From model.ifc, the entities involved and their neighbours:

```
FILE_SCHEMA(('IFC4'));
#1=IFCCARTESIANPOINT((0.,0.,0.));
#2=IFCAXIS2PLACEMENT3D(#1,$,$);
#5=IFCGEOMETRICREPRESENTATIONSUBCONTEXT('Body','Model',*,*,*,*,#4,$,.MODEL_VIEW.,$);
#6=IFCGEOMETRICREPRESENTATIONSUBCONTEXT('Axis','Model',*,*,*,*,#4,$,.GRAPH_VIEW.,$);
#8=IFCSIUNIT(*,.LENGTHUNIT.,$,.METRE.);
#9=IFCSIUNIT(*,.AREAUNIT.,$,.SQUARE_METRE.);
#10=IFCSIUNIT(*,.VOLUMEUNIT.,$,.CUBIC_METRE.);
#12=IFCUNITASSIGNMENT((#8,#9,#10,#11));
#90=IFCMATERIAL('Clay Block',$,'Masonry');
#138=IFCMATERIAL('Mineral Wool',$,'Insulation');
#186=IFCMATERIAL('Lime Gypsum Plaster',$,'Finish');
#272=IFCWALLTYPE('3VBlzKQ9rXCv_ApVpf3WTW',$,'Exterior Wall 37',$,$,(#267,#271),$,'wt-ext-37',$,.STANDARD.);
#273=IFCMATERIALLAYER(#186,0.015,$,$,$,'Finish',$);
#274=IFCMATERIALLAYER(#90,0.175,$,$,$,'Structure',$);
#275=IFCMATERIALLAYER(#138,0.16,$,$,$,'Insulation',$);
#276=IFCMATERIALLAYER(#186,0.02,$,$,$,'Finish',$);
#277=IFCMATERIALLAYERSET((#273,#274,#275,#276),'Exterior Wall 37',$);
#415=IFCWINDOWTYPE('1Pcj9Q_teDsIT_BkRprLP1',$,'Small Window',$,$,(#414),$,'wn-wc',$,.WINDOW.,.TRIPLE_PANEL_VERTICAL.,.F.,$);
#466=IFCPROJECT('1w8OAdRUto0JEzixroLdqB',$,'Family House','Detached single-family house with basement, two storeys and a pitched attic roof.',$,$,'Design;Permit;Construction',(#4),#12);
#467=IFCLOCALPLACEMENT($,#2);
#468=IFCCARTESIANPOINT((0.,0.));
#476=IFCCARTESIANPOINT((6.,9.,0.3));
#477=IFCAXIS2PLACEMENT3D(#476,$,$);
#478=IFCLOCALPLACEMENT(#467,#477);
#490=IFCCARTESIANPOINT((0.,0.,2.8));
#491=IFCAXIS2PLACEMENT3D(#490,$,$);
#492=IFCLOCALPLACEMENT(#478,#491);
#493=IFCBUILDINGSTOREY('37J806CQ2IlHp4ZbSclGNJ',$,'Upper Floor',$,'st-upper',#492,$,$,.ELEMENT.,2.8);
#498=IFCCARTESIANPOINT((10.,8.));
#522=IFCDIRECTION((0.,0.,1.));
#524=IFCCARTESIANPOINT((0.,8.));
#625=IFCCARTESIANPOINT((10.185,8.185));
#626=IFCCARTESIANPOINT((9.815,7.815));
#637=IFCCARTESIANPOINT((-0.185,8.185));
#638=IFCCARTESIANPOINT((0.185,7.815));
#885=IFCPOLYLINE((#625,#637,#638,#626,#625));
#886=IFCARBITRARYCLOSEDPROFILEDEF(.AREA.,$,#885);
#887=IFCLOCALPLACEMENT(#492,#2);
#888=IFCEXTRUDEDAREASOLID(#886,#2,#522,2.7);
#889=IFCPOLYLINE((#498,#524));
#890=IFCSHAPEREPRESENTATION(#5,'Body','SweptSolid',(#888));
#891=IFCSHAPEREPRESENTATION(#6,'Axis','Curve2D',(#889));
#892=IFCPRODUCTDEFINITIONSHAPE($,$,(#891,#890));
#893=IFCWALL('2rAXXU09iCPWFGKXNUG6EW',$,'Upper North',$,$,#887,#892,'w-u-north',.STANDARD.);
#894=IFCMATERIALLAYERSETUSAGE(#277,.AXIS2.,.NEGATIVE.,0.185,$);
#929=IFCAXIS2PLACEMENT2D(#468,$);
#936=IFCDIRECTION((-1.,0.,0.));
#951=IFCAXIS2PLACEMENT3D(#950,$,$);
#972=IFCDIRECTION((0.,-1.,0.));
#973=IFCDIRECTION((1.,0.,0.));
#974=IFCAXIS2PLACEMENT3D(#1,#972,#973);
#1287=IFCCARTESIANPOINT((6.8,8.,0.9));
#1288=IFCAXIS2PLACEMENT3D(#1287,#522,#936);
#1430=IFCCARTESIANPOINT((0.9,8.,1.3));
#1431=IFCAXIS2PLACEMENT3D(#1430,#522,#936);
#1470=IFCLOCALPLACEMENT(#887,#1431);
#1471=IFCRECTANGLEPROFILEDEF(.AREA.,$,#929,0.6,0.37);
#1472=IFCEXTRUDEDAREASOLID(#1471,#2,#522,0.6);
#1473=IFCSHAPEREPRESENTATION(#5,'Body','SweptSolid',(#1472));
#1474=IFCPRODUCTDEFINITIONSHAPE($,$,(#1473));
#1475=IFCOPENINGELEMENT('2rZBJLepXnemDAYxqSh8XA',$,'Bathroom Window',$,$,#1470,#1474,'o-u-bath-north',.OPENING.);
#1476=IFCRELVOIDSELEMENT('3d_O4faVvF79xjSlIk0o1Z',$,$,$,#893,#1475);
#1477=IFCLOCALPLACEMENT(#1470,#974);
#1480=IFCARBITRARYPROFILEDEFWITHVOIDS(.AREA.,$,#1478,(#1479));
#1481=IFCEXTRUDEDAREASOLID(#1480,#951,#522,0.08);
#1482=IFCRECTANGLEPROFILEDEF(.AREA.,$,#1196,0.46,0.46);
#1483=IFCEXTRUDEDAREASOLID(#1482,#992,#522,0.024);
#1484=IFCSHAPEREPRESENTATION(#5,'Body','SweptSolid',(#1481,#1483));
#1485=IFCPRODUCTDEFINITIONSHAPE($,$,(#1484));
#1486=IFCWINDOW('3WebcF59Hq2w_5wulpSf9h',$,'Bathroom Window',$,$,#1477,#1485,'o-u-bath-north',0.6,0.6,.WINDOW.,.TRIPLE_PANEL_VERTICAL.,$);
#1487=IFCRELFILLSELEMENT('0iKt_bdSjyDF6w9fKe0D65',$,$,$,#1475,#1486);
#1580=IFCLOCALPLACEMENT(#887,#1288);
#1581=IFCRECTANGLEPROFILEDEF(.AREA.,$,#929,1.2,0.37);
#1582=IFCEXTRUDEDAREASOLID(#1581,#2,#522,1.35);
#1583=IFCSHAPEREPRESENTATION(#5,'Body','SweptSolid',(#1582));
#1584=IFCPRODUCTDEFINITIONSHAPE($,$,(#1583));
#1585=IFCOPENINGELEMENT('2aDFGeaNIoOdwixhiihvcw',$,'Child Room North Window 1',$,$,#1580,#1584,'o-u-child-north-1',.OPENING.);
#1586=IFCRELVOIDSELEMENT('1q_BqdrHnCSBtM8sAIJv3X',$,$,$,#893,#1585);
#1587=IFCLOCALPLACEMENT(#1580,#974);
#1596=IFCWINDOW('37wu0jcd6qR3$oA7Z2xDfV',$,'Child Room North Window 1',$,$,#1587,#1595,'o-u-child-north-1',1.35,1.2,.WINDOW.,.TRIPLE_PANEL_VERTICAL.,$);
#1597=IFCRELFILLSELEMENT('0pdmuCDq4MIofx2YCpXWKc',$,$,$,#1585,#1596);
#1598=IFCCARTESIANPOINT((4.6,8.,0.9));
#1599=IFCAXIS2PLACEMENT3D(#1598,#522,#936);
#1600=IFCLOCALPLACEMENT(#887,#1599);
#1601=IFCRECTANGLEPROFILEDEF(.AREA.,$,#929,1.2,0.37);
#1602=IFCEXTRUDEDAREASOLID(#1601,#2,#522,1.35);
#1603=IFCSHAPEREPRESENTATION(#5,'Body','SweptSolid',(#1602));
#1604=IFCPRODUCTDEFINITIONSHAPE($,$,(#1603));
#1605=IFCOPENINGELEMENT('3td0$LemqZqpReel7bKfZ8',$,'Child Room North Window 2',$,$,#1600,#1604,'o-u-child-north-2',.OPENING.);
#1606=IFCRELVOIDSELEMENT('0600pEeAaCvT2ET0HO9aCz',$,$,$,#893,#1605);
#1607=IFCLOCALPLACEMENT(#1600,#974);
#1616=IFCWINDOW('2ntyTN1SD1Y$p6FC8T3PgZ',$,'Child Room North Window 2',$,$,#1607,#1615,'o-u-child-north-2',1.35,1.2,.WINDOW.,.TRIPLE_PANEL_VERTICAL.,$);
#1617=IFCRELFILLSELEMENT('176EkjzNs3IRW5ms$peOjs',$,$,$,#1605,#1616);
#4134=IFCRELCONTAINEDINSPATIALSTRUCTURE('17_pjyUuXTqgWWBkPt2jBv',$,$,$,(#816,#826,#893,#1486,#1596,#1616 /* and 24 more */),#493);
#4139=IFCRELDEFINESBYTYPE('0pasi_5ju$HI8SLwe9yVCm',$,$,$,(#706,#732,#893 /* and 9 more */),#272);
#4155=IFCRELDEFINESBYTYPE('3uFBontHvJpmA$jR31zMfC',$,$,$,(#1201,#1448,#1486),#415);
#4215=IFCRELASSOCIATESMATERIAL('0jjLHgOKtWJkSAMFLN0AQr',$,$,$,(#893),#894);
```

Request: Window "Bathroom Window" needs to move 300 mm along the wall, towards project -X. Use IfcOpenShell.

```python
import ifcopenshell
import ifcopenshell.api.geometry
import ifcopenshell.util.placement
import ifcopenshell.util.unit

model = ifcopenshell.open("model.ifc")
unit_scale = ifcopenshell.util.unit.calculate_unit_scale(model)

window = model.by_guid("3WebcF59Hq2w_5wulpSf9h")
opening = window.FillsVoids[0].RelatingOpeningElement
wall = opening.VoidsElements[0].RelatingBuildingElement

wall_matrix = ifcopenshell.util.placement.get_local_placement(wall.ObjectPlacement)
shift = wall_matrix[:3, 0] * -0.3 / unit_scale
before = ifcopenshell.util.placement.get_local_placement(window.ObjectPlacement)[:3, 3].copy()

# The window is placed relative to its opening, so it follows when the opening moves.
matrix = ifcopenshell.util.placement.get_local_placement(opening.ObjectPlacement)
matrix[:3, 3] += shift
ifcopenshell.api.geometry.edit_object_placement(
    model, product=opening, matrix=matrix, is_si=False, should_transform_children=True
)

after = ifcopenshell.util.placement.get_local_placement(window.ObjectPlacement)[:3, 3]
print("window moved by", (after - before).round(3) + 0.0)

model.write("model_edited.ifc")
```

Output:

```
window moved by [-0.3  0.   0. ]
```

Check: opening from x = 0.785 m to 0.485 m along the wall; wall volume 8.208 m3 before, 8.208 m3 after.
